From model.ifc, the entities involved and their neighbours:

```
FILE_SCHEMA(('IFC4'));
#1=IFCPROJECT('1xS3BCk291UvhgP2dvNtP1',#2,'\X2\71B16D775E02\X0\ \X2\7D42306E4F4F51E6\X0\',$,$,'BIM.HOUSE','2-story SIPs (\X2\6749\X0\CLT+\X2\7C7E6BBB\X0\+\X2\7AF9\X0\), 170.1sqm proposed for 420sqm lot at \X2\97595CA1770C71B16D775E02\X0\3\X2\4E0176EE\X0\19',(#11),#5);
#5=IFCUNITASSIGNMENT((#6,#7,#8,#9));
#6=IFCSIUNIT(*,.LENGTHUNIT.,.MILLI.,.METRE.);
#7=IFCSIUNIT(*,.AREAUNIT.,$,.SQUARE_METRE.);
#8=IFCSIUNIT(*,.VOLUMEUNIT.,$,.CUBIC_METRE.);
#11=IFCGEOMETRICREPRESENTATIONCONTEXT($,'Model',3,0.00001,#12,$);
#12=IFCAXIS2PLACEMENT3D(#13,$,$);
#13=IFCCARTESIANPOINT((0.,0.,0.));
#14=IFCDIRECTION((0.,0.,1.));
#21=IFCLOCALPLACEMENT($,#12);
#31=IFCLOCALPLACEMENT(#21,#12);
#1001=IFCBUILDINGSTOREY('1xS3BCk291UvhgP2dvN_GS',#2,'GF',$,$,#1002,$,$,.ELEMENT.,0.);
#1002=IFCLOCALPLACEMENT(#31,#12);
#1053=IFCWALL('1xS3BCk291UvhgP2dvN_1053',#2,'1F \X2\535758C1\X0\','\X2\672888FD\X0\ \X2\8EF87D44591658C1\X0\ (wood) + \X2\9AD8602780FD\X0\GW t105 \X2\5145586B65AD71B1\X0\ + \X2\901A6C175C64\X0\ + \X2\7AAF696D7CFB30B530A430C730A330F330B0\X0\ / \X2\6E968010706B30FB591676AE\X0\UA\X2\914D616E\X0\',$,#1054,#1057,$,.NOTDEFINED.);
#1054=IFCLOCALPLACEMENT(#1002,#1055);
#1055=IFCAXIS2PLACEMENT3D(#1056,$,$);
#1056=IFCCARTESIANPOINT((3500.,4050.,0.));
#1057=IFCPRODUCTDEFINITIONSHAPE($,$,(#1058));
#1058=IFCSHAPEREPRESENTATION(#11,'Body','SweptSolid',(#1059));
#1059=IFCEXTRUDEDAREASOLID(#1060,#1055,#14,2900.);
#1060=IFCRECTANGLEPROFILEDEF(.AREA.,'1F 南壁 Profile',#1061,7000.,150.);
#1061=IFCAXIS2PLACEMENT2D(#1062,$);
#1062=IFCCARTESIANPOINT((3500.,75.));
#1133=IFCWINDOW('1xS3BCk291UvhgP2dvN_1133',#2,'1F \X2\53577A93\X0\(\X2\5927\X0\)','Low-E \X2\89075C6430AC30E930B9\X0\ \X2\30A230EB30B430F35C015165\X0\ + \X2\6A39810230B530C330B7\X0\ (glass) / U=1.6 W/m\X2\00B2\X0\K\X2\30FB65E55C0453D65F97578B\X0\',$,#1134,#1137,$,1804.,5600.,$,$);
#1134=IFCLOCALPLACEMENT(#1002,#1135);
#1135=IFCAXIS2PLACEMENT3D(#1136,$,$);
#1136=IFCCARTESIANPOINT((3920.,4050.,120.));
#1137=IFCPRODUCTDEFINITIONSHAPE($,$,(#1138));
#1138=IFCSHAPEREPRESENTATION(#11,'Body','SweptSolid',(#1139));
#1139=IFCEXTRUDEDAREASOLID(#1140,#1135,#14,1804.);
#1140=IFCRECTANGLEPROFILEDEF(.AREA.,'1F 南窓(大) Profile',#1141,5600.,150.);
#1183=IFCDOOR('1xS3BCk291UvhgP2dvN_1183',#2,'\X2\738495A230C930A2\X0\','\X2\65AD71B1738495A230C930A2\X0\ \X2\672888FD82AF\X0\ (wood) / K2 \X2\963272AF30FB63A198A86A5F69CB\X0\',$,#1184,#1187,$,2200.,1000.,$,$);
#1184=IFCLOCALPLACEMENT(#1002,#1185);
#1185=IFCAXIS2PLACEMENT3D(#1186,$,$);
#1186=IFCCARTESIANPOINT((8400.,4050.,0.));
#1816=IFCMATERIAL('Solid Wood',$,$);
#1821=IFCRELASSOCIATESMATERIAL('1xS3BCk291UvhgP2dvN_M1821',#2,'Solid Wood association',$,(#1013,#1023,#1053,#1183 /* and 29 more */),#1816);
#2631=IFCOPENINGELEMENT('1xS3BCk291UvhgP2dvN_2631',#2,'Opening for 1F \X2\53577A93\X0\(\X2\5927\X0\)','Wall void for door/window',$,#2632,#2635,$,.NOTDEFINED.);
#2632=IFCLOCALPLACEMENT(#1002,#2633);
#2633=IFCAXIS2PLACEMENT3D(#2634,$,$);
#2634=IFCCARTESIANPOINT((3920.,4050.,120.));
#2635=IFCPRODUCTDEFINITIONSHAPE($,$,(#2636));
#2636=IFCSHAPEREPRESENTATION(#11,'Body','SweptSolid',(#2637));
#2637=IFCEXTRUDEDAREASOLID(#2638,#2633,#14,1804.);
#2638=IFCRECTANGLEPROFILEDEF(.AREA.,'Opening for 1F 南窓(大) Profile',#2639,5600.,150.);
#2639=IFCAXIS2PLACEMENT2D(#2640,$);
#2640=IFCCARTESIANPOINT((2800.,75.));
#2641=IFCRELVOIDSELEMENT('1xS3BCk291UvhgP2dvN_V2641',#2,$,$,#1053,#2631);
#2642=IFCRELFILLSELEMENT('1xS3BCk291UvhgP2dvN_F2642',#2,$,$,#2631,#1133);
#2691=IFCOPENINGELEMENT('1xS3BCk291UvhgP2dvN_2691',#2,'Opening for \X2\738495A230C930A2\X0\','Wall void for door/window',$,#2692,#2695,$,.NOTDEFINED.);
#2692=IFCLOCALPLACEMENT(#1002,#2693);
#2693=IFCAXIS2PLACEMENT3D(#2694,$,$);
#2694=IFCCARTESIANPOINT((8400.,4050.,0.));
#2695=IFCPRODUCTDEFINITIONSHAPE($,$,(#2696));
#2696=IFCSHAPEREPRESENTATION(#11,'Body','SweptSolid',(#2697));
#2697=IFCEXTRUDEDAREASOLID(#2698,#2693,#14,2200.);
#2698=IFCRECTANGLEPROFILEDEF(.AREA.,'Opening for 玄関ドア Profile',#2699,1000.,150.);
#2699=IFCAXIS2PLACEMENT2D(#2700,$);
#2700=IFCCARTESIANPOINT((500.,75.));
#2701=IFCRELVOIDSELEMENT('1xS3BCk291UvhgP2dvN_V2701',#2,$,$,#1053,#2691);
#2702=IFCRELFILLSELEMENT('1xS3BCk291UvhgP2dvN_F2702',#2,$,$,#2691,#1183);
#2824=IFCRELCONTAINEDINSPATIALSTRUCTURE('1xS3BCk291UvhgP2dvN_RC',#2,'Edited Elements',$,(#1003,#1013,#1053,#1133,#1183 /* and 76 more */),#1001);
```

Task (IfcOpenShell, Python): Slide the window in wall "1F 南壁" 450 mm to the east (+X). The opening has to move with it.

```python
import ifcopenshell
import ifcopenshell.api.geometry
import ifcopenshell.util.placement
import ifcopenshell.util.unit

model = ifcopenshell.open("model.ifc")
unit_scale = ifcopenshell.util.unit.calculate_unit_scale(model)

window = model.by_guid("1xS3BCk291UvhgP2dvN_1133")
opening = window.FillsVoids[0].RelatingOpeningElement
wall = opening.VoidsElements[0].RelatingBuildingElement

wall_matrix = ifcopenshell.util.placement.get_local_placement(wall.ObjectPlacement)
shift = wall_matrix[:3, 0] * 0.45 / unit_scale
before = ifcopenshell.util.placement.get_local_placement(window.ObjectPlacement)[:3, 3].copy()

# The window is not placed relative to its opening, so move both.
for product in (opening, window):
    matrix = ifcopenshell.util.placement.get_local_placement(product.ObjectPlacement)
    matrix[:3, 3] += shift
    ifcopenshell.api.geometry.edit_object_placement(model, product=product, matrix=matrix, is_si=False)

after = ifcopenshell.util.placement.get_local_placement(window.ObjectPlacement)[:3, 3]
print("window moved by", (after - before).round(3) + 0.0)

model.write("model_rev.ifc")
```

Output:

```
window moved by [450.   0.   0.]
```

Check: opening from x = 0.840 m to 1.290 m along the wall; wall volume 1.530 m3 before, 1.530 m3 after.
